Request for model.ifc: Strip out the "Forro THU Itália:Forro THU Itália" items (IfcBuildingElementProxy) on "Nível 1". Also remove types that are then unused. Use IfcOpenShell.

First a look at what the model holds.

```python
import ifcopenshell
import ifcopenshell.util.element

model = ifcopenshell.open("model.ifc")
print(model.schema)
storey = next(s for s in model.by_type("IfcBuildingStorey") if s.Name == "Nível 1")
proxies = [e for e in ifcopenshell.util.element.get_decomposition(storey) if e.is_a("IfcBuildingElementProxy")]
seen = {}
for e in proxies:
    element_type = ifcopenshell.util.element.get_type(e)
    name = element_type.Name if element_type not in (None, e) else None
    seen[name] = seen.get(name, 0) + 1
for name, count in sorted(seen.items(), key=str):
    print(count, "x", name)
```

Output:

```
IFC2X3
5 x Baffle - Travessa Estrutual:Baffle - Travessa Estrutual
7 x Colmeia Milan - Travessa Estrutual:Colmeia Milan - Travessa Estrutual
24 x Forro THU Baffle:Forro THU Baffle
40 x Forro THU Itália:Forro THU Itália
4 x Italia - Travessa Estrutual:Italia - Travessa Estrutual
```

```python
import ifcopenshell
import ifcopenshell.api.root
import ifcopenshell.util.element

model = ifcopenshell.open("model.ifc")

storey = next(s for s in model.by_type("IfcBuildingStorey") if s.Name == "Nível 1")
proxies = [e for e in ifcopenshell.util.element.get_decomposition(storey) if e.is_a("IfcBuildingElementProxy")]
targets = [e for e in proxies if (t := ifcopenshell.util.element.get_type(e)) not in (None, e) and t.Name == "Forro THU Itália:Forro THU Itália"]
types = {ifcopenshell.util.element.get_type(e) for e in targets} - {None, *targets}

for e in targets:
    ifcopenshell.api.root.remove_product(model, product=e)
print(len(targets), "removed")

unused = [t for t in types if not ifcopenshell.util.element.get_types(t)]
for t in unused:
    ifcopenshell.api.root.remove_product(model, product=t)
print(len(unused), "unused types removed")

model.write("model_rev.ifc")
```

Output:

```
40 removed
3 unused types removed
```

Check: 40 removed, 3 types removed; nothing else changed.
